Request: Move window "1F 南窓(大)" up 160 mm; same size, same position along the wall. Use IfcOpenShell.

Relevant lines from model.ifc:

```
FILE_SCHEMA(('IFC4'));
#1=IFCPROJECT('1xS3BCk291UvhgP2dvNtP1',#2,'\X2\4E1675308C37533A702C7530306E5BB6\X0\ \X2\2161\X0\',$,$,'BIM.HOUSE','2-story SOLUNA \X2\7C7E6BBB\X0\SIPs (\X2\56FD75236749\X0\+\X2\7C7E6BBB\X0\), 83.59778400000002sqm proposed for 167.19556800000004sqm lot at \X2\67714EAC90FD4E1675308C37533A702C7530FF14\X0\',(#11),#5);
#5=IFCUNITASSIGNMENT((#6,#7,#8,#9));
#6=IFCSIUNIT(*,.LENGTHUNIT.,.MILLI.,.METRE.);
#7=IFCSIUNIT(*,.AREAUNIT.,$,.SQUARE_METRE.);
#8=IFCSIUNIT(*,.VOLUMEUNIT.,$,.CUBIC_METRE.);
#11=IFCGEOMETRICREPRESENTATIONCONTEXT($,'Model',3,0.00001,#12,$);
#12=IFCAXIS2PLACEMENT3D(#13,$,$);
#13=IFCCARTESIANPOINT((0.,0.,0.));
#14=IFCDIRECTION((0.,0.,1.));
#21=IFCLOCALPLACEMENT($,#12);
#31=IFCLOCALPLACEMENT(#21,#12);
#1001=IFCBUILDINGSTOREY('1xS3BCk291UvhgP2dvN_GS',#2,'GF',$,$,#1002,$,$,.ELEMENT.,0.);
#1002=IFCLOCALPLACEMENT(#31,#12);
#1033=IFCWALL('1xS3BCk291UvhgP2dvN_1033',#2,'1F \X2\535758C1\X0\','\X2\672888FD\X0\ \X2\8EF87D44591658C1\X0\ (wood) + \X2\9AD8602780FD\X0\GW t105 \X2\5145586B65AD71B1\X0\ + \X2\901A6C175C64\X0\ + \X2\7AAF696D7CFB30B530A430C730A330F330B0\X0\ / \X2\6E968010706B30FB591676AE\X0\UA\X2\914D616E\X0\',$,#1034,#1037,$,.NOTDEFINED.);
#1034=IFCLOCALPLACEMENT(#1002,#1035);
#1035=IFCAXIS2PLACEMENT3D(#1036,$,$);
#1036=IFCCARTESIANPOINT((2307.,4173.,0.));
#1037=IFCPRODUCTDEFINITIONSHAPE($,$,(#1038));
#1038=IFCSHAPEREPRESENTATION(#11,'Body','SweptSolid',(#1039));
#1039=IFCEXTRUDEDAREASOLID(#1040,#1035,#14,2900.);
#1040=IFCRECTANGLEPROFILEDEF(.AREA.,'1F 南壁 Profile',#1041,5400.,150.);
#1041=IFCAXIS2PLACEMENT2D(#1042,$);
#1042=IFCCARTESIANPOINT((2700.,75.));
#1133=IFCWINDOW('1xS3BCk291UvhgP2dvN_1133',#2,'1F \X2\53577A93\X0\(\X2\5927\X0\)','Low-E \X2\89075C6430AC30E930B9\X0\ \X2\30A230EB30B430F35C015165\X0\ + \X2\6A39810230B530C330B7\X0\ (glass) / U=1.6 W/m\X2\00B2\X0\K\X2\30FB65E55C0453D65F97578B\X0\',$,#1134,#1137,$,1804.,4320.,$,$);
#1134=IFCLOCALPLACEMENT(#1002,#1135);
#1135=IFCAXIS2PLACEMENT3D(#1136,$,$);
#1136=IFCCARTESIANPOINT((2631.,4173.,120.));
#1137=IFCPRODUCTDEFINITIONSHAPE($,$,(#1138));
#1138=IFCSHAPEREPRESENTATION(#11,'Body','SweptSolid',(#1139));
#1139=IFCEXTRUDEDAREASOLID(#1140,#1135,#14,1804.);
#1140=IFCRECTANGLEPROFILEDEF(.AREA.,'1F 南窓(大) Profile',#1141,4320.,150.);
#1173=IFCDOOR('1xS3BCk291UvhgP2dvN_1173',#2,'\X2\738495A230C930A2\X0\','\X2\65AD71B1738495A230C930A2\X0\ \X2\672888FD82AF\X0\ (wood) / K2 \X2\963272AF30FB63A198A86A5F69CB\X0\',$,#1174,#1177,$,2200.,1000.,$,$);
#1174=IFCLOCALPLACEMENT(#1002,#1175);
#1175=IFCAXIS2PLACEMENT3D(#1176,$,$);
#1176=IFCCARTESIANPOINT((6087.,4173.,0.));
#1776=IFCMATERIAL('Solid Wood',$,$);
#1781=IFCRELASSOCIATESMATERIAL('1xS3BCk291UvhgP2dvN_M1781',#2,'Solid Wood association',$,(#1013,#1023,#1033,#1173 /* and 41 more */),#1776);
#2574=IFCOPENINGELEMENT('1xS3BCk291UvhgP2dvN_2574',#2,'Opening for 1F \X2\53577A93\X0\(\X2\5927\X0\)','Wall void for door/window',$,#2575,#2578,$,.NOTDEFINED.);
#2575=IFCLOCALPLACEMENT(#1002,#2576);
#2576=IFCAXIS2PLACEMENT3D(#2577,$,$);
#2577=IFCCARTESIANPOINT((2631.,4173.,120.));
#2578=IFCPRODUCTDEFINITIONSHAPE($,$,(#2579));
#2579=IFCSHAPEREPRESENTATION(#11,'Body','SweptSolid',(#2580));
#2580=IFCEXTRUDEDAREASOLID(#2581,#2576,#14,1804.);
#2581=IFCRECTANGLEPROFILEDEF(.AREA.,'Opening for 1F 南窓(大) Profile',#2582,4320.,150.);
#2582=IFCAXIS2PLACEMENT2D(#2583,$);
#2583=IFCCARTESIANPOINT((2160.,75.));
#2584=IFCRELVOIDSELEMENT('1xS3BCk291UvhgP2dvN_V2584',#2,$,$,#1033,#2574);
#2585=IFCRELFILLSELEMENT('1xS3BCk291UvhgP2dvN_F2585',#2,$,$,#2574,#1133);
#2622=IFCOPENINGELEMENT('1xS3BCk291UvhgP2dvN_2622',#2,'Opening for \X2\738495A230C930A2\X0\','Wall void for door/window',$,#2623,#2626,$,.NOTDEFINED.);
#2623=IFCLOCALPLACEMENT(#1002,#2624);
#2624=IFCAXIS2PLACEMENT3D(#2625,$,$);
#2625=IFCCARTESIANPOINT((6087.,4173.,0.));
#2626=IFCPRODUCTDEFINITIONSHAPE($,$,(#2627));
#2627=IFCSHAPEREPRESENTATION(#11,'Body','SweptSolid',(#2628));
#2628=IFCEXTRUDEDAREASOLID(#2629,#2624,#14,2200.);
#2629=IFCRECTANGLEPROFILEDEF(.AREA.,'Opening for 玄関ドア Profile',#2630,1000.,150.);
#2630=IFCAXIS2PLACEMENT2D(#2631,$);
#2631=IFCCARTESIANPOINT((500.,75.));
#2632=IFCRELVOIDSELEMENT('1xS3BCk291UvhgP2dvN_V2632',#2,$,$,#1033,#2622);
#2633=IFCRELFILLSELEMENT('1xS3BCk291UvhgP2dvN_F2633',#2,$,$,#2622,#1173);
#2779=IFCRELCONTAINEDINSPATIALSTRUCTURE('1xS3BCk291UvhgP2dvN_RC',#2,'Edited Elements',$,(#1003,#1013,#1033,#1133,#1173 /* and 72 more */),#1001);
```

```python
import numpy as np
import ifcopenshell
import ifcopenshell.api.geometry
import ifcopenshell.util.placement
import ifcopenshell.util.unit

model = ifcopenshell.open("model.ifc")
unit_scale = ifcopenshell.util.unit.calculate_unit_scale(model)

window = model.by_id(1133)
opening = window.FillsVoids[0].RelatingOpeningElement
dz = 0.16 / unit_scale

shift = np.array([0.0, 0.0, dz])
# The window is not placed relative to its opening, so move both.
for product in (opening, window):
    matrix = ifcopenshell.util.placement.get_local_placement(product.ObjectPlacement)
    matrix[:3, 3] += shift
    ifcopenshell.api.geometry.edit_object_placement(model, product=product, matrix=matrix, is_si=False)

print(f"moved by {dz * unit_scale:+.3f} m")

model.write("model-out.ifc")
```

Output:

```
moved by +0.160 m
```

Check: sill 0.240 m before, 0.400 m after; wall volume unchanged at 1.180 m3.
